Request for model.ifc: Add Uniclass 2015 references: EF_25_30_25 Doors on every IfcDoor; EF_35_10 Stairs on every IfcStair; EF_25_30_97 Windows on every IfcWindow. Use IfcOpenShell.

First a look at what the model holds.

```python
import ifcopenshell

model = ifcopenshell.open("model.ifc")
print(model.schema)
print("classifications:", [c.Name for c in model.by_type("IfcClassification")])
for ifc_class in ("IfcDoor", "IfcRoof", "IfcStair", "IfcWall", "IfcWindow"):
    print(ifc_class, len(model.by_type(ifc_class)))
```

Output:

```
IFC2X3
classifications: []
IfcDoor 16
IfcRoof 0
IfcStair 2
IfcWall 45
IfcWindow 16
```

```python
import ifcopenshell
import ifcopenshell.api.classification

model = ifcopenshell.open("model.ifc")

# IFC2X3 requires Source and Edition and has no link from the project to the system.
system = model.create_entity("IfcClassification", Source="NBS", Edition="2015", Name="Uniclass 2015")

codes = {
    "IfcDoor": ("EF_25_30_25", "Doors"),
    "IfcStair": ("EF_35_10", "Stairs"),
    "IfcWindow": ("EF_25_30_97", "Windows"),
}
for ifc_class, (code, name) in codes.items():
    products = model.by_type(ifc_class)
    ifcopenshell.api.classification.add_reference(
        model, products=products, classification=system, identification=code, name=name
    )
    print(code, len(products))

model.write("model_updated.ifc")
```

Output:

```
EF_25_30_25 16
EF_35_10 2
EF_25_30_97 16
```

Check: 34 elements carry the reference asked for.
